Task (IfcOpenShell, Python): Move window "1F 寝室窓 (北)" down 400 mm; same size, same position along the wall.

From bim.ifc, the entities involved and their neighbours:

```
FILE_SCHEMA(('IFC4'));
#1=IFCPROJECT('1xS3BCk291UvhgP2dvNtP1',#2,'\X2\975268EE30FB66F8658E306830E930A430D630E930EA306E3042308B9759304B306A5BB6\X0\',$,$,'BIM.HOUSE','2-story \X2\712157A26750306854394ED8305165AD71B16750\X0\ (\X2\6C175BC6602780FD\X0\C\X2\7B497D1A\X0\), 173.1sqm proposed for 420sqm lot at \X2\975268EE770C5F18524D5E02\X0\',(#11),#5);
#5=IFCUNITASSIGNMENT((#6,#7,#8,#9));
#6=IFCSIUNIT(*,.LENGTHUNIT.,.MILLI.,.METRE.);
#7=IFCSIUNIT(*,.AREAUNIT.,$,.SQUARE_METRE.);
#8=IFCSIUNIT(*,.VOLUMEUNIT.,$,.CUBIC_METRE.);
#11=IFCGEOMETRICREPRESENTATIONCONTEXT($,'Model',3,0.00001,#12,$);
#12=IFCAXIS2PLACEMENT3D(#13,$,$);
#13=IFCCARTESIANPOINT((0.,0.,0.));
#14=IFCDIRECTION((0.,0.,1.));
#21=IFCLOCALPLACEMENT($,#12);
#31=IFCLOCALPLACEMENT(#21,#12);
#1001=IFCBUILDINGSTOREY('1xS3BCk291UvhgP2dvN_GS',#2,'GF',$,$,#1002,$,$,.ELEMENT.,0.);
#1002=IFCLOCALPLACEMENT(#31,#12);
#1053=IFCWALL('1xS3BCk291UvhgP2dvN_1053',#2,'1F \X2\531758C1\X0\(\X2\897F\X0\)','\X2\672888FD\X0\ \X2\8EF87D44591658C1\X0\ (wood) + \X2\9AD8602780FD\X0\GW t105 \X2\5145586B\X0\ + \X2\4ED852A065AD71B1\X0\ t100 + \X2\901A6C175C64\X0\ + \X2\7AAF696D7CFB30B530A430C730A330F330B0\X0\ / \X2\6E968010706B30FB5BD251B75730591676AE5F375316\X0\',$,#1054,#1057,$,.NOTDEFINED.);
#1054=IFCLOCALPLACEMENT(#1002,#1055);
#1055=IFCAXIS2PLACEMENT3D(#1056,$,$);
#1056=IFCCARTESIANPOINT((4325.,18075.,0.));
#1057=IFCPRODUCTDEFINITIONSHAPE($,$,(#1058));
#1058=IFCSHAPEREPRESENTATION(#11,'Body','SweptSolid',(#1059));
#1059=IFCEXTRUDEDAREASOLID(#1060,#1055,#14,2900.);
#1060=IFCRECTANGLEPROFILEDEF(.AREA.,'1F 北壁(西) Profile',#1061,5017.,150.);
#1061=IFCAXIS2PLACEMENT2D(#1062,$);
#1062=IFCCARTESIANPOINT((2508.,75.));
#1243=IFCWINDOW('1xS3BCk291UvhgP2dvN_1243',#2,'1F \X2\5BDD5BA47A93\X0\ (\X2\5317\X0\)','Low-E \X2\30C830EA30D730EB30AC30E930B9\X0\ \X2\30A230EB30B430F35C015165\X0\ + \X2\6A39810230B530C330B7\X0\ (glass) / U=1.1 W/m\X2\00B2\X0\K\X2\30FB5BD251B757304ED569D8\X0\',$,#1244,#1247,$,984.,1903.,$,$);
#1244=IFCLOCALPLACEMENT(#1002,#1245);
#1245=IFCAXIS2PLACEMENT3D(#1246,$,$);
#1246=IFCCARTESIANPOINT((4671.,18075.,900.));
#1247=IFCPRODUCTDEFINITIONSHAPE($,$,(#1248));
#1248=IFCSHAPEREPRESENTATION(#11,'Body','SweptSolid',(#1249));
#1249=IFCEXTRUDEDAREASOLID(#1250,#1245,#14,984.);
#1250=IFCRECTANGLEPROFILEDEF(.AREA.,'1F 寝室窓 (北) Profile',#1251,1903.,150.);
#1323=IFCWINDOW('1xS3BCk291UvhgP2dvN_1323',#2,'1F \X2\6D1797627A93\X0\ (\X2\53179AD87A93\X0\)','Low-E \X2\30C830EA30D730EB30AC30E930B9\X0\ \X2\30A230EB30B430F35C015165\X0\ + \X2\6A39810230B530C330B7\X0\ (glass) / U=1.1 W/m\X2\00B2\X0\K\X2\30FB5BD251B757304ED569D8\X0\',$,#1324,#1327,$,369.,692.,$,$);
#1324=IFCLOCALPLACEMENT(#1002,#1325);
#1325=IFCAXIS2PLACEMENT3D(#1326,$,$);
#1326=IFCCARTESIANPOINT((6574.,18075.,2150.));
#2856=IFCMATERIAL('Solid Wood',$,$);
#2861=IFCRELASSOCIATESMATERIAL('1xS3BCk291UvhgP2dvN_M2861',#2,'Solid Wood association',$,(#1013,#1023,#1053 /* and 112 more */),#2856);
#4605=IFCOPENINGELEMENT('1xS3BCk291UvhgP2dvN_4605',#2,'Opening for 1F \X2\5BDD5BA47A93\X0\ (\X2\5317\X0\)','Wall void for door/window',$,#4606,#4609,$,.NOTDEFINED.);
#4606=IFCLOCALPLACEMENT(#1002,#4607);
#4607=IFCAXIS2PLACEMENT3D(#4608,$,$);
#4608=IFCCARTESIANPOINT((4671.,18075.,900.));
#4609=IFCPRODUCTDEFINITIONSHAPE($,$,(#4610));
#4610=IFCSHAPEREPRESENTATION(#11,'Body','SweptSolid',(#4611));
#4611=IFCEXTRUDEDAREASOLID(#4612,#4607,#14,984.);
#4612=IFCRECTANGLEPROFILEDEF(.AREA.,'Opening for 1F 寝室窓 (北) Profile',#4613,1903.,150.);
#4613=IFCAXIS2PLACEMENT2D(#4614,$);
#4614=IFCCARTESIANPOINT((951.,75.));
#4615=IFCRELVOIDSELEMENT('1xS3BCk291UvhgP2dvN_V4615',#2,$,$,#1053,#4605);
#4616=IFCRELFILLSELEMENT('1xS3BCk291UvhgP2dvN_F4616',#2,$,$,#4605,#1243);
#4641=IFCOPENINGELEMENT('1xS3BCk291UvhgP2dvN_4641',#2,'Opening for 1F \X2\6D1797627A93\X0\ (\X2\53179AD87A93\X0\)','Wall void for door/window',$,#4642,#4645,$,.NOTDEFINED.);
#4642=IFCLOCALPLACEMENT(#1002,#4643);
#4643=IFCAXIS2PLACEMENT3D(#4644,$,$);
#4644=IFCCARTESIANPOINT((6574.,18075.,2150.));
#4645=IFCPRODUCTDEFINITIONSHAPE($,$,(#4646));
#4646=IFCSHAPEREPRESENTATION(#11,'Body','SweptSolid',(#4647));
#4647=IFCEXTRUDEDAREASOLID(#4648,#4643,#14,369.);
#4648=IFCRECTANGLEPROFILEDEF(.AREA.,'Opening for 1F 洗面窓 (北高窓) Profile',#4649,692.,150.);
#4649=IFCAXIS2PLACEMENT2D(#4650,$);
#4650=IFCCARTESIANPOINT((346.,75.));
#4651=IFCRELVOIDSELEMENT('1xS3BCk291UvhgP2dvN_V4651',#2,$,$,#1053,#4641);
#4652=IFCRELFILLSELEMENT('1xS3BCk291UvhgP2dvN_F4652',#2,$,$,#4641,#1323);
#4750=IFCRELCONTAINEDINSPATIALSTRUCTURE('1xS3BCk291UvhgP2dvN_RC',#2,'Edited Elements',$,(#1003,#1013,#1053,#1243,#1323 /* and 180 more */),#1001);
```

```python
import numpy as np
import ifcopenshell
import ifcopenshell.api.geometry
import ifcopenshell.util.placement
import ifcopenshell.util.unit

model = ifcopenshell.open("bim.ifc")
unit_scale = ifcopenshell.util.unit.calculate_unit_scale(model)

window = model.by_guid("1xS3BCk291UvhgP2dvN_1243")
opening = window.FillsVoids[0].RelatingOpeningElement
dz = -0.4 / unit_scale

shift = np.array([0.0, 0.0, dz])
# The window is not placed relative to its opening, so move both.
for product in (opening, window):
    matrix = ifcopenshell.util.placement.get_local_placement(product.ObjectPlacement)
    matrix[:3, 3] += shift
    ifcopenshell.api.geometry.edit_object_placement(model, product=product, matrix=matrix, is_si=False)

print(f"moved by {dz * unit_scale:+.3f} m")

model.write("bim_edited.ifc")
```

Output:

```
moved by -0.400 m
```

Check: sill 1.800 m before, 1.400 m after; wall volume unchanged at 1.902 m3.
